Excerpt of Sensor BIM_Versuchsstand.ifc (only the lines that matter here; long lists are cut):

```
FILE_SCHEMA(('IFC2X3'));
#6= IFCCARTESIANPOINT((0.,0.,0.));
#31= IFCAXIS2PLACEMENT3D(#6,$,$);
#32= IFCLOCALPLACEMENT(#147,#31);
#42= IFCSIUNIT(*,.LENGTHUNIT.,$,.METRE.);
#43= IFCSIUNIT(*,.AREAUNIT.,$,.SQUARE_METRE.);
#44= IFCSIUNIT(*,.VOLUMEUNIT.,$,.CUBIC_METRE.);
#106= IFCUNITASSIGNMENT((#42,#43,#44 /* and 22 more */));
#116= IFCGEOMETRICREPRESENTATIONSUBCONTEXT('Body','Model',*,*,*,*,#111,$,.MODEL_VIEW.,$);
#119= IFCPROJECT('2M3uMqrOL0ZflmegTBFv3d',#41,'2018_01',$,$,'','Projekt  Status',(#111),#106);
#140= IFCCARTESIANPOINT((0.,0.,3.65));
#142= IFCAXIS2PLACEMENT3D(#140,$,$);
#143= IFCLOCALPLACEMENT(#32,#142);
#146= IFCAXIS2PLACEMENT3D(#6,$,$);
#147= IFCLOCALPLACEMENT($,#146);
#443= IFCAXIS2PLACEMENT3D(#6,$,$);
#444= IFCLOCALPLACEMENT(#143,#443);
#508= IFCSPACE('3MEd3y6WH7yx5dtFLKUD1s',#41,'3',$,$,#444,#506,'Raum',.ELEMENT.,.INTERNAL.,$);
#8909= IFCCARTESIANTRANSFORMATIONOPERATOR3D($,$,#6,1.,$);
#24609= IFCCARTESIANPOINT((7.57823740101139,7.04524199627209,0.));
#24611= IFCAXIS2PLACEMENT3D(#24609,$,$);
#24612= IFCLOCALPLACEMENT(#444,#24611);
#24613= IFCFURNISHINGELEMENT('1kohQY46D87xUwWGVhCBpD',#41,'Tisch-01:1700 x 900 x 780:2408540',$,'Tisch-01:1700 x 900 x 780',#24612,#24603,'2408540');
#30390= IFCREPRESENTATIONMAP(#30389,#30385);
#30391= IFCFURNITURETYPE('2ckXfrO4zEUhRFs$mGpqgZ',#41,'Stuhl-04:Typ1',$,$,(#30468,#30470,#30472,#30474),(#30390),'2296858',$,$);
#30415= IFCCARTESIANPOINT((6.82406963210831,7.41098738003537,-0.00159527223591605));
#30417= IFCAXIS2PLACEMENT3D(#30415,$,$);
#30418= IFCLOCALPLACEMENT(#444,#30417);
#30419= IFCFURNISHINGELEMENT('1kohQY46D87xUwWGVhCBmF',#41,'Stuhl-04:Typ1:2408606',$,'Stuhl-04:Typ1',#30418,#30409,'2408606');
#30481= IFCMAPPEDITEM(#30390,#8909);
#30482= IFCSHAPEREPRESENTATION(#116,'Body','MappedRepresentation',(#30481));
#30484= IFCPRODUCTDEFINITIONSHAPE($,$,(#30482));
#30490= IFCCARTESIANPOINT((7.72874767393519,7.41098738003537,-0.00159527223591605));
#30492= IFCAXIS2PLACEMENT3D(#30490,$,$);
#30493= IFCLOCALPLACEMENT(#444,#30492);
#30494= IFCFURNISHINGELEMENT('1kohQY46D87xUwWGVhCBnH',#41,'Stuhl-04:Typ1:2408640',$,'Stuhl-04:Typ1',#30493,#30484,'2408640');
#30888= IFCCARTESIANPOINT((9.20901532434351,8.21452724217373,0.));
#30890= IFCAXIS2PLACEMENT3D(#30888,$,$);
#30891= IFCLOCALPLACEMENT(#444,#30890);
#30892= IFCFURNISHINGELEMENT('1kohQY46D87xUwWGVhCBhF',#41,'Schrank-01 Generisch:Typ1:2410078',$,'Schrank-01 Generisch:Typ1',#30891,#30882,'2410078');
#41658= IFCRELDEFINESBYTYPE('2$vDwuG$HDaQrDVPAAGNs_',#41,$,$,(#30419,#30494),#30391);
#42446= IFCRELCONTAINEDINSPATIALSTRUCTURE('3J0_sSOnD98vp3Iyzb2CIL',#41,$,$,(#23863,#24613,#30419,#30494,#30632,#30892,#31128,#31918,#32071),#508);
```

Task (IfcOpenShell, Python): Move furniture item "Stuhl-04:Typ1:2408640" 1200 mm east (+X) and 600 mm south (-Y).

```python
import ifcopenshell
import ifcopenshell.api.geometry
import ifcopenshell.util.placement

model = ifcopenshell.open("Sensor BIM_Versuchsstand.ifc")

item = model.by_guid("1kohQY46D87xUwWGVhCBnH")
matrix = ifcopenshell.util.placement.get_local_placement(item.ObjectPlacement)
matrix[0, 3] += 1.2
matrix[1, 3] -= 0.6
ifcopenshell.api.geometry.edit_object_placement(model, product=item, matrix=matrix, is_si=False)

print(ifcopenshell.util.placement.get_local_placement(item.ObjectPlacement).round(3) + 0.0)

model.write("Sensor BIM_Versuchsstand_edited.ifc")
```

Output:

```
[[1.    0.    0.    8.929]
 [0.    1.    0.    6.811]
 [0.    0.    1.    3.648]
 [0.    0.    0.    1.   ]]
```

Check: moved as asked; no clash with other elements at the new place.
